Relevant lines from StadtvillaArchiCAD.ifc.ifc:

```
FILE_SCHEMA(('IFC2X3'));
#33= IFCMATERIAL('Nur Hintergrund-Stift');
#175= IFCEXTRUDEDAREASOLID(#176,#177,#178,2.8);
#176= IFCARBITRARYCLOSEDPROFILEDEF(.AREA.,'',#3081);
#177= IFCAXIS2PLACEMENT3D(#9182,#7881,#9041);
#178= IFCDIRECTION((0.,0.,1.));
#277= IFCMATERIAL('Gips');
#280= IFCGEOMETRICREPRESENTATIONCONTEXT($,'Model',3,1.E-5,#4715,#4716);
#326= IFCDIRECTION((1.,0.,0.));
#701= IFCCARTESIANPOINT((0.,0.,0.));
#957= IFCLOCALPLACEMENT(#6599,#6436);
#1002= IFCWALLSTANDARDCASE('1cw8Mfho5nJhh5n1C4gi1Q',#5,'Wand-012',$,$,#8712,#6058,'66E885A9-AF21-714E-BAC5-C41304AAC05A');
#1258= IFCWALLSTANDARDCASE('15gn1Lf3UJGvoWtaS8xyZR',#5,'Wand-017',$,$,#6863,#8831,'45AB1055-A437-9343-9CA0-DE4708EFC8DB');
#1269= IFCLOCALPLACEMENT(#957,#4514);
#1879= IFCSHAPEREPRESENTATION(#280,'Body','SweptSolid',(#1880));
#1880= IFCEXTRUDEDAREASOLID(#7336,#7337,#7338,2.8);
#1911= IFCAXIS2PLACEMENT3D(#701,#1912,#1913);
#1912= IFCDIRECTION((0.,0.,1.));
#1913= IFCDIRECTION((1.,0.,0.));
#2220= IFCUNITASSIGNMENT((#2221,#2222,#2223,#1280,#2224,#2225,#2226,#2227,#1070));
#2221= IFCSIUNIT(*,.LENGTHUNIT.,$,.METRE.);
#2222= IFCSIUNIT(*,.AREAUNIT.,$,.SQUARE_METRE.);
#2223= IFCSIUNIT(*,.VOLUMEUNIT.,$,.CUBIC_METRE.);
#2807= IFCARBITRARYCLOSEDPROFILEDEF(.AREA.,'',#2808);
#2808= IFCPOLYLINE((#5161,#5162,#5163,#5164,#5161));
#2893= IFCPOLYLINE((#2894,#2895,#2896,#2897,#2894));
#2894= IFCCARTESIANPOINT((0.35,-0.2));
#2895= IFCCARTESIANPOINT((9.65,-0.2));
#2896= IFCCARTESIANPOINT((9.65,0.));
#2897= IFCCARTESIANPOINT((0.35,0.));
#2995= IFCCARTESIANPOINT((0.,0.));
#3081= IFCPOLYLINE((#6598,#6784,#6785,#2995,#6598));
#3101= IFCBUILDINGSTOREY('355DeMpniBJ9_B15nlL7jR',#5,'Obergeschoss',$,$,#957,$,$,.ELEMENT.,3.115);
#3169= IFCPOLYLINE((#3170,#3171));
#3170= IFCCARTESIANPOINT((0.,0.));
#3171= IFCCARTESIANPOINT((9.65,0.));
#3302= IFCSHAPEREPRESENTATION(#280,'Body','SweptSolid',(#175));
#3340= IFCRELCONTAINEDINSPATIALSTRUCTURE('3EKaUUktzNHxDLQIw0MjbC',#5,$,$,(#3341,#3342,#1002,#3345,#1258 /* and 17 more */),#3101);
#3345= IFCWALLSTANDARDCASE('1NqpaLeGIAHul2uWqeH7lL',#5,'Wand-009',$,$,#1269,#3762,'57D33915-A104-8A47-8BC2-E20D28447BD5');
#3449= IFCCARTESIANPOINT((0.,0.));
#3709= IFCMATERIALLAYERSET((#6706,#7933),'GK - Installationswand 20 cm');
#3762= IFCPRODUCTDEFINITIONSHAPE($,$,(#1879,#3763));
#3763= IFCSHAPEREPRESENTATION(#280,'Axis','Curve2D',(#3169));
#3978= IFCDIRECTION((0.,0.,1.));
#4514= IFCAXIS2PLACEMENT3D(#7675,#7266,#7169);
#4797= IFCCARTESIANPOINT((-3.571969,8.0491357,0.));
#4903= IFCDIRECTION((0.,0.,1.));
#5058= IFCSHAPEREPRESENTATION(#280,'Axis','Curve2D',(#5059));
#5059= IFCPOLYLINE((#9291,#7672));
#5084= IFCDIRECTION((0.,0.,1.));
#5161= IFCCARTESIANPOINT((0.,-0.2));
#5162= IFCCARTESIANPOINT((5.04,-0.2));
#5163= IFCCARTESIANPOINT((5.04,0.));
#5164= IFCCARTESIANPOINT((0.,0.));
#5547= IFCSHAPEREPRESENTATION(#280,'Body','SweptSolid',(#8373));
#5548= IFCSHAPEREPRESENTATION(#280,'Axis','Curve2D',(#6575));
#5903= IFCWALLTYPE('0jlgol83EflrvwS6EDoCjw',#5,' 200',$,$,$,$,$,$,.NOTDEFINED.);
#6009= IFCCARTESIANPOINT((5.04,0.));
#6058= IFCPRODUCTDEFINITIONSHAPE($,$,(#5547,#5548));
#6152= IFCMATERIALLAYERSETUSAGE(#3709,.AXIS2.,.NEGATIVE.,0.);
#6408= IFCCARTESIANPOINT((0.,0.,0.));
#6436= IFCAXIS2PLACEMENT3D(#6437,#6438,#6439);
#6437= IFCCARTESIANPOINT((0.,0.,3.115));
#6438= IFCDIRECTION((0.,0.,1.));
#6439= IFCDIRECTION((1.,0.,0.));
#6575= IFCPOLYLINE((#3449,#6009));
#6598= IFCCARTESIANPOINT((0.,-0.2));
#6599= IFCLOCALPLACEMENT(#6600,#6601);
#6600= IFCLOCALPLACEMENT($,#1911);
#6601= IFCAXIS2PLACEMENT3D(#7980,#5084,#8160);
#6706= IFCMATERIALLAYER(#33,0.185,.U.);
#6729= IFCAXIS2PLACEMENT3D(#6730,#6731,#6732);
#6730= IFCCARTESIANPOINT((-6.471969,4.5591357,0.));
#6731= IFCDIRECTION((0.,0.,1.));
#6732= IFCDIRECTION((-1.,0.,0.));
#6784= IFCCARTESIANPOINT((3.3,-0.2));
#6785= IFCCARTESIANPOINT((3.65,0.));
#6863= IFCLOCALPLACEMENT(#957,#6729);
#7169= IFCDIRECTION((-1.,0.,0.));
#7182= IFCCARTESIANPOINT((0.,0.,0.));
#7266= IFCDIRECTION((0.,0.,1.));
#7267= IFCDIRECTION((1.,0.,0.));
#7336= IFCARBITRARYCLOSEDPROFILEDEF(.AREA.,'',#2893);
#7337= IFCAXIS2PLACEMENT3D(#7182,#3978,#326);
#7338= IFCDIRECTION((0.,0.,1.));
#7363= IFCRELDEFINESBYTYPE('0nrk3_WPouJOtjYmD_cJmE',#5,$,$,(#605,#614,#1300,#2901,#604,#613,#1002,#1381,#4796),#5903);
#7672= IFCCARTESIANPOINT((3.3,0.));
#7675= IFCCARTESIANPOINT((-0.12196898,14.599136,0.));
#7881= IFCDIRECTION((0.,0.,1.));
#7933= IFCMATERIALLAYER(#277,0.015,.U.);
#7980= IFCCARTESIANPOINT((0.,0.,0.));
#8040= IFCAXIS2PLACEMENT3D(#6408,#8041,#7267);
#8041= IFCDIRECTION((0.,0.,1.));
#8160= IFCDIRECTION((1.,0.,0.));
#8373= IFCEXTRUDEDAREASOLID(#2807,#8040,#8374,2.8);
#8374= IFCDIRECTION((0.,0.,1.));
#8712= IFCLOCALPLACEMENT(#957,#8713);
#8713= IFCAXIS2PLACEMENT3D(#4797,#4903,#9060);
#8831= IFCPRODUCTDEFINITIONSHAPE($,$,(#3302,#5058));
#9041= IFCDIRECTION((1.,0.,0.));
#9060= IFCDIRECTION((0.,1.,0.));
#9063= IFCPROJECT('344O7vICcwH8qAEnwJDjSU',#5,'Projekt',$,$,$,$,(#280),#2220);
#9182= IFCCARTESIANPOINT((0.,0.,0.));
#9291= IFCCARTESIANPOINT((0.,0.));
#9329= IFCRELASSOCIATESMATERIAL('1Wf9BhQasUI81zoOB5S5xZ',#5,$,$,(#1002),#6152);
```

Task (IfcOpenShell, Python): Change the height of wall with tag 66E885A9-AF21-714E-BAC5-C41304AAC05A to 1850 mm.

```python
import ifcopenshell
import ifcopenshell.geom
import ifcopenshell.util.shape
import ifcopenshell.util.unit

model = ifcopenshell.open("StadtvillaArchiCAD.ifc.ifc")
unit_scale = ifcopenshell.util.unit.calculate_unit_scale(model)
settings = ifcopenshell.geom.settings()


def volume(element):
    """Net volume in cubic metres, openings subtracted."""
    shape = ifcopenshell.geom.create_shape(settings, element)
    return ifcopenshell.util.shape.get_volume(shape.geometry)


wall = model.by_guid("1cw8Mfho5nJhh5n1C4gi1Q")
before = volume(wall)

body = next(r for r in wall.Representation.Representations if r.RepresentationIdentifier == "Body")
solid = body.Items[0]
old_height = solid.Depth
solid.Depth = 1.85 / unit_scale
after = volume(wall)

print(f"height {old_height:g} -> {solid.Depth:g}, volume {before:.3f} -> {after:.3f} m3")

model.write("StadtvillaArchiCAD.ifc_updated.ifc")
```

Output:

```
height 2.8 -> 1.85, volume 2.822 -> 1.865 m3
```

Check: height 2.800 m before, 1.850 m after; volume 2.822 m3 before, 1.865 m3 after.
